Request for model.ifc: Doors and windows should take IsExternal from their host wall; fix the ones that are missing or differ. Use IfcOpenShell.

First a look at what the model holds.

```python
import ifcopenshell
import ifcopenshell.util.element

model = ifcopenshell.open("model.ifc")
print(model.schema)
seen = {}
for e in model.by_type("IfcDoor") + model.by_type("IfcWindow"):
    if not e.FillsVoids:
        continue
    host = e.FillsVoids[0].RelatingOpeningElement.VoidsElements[0].RelatingBuildingElement
    own = ifcopenshell.util.element.get_pset(e, f"Pset_{e.is_a()[3:].removesuffix('StandardCase')}Common", "IsExternal")
    wall = ifcopenshell.util.element.get_pset(host, "Pset_WallCommon", "IsExternal")
    seen[e.is_a(), own, wall] = seen.get((e.is_a(), own, wall), 0) + 1
for (cls, own, wall), count in sorted(seen.items(), key=str):
    print(count, cls, "IsExternal:", own, "| host wall:", wall)
```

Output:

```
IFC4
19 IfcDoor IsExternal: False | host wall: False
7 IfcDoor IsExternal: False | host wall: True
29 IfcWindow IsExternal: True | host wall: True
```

```python
import ifcopenshell
import ifcopenshell.api.pset
import ifcopenshell.util.element

model = ifcopenshell.open("model.ifc")

count = 0
for ifc_class, pset_name in (("IfcDoor", "Pset_DoorCommon"), ("IfcWindow", "Pset_WindowCommon")):
    for e in model.by_type(ifc_class):
        if not e.FillsVoids:
            continue
        host = e.FillsVoids[0].RelatingOpeningElement.VoidsElements[0].RelatingBuildingElement
        external = ifcopenshell.util.element.get_pset(host, "Pset_WallCommon", "IsExternal")
        if external is None or ifcopenshell.util.element.get_pset(e, pset_name, "IsExternal") == external:
            continue
        pset = ifcopenshell.api.pset.add_pset(model, product=e, name=pset_name)
        ifcopenshell.api.pset.edit_pset(model, pset=pset, properties={"IsExternal": external})
        count += 1

print(count, "updated")

model.write("model_updated.ifc")
```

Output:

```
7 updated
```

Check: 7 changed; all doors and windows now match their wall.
